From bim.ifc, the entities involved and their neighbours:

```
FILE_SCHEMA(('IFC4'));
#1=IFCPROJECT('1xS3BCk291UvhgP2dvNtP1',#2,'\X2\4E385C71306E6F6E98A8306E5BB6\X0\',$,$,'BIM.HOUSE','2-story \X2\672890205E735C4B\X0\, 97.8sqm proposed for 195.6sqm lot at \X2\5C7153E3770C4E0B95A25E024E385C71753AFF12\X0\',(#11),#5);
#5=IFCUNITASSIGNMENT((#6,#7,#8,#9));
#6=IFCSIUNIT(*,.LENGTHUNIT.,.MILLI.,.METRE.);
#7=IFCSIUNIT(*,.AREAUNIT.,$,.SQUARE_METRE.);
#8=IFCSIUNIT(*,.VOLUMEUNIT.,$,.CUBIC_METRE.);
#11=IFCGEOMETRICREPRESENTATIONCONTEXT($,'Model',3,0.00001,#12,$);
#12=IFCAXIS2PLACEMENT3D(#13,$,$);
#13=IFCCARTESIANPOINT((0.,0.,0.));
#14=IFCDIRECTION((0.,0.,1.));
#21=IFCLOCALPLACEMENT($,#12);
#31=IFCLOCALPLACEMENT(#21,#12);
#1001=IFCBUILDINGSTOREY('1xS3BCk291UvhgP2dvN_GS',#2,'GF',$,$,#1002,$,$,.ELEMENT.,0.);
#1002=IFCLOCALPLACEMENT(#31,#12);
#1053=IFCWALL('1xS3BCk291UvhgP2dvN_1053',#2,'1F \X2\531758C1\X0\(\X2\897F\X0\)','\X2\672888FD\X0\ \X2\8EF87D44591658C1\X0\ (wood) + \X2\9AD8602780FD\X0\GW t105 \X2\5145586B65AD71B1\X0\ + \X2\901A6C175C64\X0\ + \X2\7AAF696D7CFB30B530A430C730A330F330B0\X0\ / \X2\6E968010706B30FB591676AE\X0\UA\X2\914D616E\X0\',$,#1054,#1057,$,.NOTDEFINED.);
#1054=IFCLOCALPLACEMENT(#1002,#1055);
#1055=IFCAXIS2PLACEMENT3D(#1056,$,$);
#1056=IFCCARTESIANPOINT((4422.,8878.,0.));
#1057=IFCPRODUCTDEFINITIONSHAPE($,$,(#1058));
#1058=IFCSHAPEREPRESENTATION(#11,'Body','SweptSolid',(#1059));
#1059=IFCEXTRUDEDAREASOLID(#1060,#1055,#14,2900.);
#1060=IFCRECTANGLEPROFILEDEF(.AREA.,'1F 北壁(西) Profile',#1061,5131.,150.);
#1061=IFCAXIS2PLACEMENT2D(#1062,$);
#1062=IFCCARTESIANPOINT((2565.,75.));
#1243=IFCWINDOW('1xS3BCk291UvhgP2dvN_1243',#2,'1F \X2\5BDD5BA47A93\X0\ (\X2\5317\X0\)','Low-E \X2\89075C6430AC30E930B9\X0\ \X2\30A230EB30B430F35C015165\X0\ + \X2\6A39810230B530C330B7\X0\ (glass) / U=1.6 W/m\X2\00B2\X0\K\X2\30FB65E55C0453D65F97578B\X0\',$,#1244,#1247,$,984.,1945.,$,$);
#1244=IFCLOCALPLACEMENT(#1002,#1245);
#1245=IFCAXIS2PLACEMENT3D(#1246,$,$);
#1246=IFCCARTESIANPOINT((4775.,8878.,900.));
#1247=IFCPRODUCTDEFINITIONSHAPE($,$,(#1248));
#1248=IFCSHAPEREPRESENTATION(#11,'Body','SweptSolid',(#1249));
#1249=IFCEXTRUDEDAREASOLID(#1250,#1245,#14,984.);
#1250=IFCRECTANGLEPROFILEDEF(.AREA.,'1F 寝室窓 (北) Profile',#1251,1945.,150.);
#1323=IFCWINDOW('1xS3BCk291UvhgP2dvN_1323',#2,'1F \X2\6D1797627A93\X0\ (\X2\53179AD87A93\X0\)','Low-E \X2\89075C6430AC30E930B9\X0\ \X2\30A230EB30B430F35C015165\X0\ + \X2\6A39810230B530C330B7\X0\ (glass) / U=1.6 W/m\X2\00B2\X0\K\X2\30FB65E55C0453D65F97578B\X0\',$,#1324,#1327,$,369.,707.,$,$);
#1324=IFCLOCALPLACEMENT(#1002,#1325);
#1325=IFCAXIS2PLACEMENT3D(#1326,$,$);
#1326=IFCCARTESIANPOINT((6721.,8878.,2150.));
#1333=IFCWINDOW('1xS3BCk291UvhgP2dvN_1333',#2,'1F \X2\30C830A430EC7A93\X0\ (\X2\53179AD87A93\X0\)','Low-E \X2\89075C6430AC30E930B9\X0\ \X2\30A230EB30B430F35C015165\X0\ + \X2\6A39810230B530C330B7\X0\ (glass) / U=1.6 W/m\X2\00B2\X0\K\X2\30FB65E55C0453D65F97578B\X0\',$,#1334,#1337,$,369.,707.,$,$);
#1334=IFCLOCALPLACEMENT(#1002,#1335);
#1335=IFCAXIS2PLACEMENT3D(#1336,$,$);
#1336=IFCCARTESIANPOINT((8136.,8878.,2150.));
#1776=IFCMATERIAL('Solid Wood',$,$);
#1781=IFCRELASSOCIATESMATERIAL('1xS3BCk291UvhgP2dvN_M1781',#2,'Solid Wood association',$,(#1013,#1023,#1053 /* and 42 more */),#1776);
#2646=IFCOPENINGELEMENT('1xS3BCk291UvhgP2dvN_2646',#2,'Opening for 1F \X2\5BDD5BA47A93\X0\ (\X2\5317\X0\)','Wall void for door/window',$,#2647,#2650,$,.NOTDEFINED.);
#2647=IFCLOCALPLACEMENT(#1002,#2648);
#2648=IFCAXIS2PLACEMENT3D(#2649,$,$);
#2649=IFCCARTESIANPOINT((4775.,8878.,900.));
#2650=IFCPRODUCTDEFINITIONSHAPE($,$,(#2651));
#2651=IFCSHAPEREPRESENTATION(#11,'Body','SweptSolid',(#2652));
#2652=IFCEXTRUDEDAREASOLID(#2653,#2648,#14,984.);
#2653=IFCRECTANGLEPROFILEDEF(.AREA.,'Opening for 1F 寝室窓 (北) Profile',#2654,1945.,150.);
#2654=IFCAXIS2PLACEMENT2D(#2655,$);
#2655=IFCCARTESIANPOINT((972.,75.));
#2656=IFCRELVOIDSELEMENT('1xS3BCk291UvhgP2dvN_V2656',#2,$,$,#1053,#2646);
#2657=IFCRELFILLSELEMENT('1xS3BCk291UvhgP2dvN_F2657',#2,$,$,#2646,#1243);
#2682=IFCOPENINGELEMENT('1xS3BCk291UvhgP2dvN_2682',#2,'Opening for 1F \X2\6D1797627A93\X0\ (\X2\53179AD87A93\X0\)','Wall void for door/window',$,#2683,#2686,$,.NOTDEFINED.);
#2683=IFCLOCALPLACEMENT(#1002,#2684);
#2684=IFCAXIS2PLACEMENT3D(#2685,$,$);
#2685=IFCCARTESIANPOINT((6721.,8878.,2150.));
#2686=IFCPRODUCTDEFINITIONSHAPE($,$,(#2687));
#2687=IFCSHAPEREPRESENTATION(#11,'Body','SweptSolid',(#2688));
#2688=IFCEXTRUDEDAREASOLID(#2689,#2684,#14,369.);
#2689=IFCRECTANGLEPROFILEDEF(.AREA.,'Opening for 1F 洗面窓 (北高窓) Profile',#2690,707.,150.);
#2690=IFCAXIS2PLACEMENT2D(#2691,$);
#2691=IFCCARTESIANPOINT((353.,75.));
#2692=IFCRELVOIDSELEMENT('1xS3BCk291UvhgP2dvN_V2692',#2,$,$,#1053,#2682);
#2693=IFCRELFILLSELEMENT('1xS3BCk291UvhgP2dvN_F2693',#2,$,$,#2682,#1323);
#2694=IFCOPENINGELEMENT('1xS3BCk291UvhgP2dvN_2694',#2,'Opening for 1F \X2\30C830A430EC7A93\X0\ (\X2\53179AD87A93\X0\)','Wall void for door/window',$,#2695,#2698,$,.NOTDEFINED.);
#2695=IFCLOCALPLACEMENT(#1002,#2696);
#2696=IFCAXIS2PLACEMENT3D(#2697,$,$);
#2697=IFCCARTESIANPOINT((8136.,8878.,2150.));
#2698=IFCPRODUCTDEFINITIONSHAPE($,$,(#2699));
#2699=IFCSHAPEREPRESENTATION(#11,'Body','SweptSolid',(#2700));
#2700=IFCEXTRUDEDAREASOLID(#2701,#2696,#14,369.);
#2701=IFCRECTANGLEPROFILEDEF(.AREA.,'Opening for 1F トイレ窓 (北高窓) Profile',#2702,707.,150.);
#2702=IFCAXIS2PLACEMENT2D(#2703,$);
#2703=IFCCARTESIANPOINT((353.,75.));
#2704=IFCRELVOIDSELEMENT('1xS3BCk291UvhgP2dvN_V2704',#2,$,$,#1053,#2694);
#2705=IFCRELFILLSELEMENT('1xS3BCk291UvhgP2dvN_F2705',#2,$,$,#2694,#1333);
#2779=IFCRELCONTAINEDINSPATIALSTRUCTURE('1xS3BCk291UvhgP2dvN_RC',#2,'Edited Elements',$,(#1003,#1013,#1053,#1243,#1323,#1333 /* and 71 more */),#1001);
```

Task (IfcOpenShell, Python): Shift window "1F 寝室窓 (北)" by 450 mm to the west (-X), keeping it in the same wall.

```python
import ifcopenshell
import ifcopenshell.api.geometry
import ifcopenshell.util.placement

model = ifcopenshell.open("bim.ifc")

window = model.by_guid("1xS3BCk291UvhgP2dvN_1243")
opening = window.FillsVoids[0].RelatingOpeningElement
wall = opening.VoidsElements[0].RelatingBuildingElement

wall_matrix = ifcopenshell.util.placement.get_local_placement(wall.ObjectPlacement)
shift = wall_matrix[:3, 0] * -450.0
before = ifcopenshell.util.placement.get_local_placement(window.ObjectPlacement)[:3, 3].copy()

# The window is not placed relative to its opening, so move both.
for product in (opening, window):
    matrix = ifcopenshell.util.placement.get_local_placement(product.ObjectPlacement)
    matrix[:3, 3] += shift
    ifcopenshell.api.geometry.edit_object_placement(model, product=product, matrix=matrix, is_si=False)

after = ifcopenshell.util.placement.get_local_placement(window.ObjectPlacement)[:3, 3]
print("window moved by", (after - before).round(3) + 0.0)

model.write("bim_rev.ifc")
```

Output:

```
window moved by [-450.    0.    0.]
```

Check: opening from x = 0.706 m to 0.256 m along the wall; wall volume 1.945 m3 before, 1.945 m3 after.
